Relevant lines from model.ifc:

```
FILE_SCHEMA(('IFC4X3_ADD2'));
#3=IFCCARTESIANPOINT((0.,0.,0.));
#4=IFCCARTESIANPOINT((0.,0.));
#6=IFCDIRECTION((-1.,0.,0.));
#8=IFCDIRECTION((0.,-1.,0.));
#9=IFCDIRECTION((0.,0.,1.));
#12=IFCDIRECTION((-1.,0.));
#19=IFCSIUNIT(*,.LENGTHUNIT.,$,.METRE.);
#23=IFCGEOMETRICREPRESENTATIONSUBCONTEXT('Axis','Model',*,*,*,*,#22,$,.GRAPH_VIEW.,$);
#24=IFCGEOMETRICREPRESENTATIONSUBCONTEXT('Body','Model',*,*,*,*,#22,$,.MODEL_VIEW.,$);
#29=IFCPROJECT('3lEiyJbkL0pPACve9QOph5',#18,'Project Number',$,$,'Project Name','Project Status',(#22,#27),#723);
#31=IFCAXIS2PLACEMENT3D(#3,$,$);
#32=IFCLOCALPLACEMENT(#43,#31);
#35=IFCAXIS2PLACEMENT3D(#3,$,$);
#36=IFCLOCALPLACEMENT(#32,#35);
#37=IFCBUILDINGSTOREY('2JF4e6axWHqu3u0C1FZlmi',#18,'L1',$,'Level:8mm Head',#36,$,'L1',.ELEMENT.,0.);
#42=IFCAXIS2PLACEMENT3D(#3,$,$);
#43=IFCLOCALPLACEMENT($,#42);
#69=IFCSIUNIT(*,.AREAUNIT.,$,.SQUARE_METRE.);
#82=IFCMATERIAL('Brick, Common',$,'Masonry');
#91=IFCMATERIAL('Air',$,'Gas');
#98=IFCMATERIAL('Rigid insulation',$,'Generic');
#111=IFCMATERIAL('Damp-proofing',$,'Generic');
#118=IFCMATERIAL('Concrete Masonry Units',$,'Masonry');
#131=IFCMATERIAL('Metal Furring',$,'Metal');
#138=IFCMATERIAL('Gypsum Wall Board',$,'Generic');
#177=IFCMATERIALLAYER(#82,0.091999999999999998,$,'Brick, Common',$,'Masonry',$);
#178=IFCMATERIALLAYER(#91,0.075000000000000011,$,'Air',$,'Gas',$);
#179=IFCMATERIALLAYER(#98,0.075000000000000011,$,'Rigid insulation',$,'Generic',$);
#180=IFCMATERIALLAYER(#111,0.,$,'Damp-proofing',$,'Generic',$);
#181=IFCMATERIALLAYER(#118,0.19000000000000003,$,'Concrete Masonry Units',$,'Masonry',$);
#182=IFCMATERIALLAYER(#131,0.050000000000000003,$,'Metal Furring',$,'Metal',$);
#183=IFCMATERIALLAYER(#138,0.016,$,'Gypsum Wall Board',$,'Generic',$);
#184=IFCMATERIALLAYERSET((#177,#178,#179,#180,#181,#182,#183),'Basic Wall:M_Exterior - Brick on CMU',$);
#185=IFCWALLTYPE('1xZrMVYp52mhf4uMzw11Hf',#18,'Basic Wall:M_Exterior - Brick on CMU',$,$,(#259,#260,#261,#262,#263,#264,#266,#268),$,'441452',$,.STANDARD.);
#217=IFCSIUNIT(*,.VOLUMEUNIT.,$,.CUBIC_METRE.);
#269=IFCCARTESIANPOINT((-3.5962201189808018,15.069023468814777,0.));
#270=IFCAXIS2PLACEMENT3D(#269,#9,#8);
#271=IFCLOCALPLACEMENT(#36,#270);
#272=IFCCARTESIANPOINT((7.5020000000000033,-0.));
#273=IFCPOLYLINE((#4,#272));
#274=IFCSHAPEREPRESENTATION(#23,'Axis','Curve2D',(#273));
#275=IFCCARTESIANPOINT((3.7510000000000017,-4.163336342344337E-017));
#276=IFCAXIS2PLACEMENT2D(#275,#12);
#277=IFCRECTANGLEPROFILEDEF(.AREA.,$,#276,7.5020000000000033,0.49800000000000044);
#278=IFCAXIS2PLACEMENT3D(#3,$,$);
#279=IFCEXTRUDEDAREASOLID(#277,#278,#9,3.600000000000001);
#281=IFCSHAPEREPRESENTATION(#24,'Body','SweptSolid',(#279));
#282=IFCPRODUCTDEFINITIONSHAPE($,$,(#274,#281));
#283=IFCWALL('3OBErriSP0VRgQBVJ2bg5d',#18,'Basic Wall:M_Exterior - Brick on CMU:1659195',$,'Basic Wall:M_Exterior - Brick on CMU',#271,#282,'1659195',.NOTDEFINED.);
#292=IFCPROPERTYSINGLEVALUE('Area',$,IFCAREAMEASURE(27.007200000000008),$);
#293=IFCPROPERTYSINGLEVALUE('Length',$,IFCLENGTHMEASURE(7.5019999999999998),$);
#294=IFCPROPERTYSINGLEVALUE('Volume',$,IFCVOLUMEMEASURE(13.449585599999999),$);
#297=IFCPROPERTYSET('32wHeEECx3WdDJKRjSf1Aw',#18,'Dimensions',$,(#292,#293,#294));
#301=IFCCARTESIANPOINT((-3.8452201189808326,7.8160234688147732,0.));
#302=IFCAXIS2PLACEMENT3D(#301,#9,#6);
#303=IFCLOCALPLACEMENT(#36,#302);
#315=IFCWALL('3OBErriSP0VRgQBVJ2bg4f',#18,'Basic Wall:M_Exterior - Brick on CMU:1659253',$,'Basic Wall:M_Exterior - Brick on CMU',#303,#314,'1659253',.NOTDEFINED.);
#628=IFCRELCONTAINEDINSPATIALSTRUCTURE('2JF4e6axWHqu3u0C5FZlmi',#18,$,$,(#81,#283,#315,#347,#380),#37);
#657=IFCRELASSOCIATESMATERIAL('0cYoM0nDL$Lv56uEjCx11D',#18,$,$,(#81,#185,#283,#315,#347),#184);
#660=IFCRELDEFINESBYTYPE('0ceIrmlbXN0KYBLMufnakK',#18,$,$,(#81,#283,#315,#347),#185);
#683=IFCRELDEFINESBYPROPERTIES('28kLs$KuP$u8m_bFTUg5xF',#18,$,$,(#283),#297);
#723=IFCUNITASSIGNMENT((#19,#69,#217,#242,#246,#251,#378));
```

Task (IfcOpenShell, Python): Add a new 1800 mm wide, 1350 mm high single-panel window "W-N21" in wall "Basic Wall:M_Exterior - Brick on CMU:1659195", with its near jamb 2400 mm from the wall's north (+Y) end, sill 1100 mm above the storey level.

```python
import numpy as np
import ifcopenshell
import ifcopenshell.api.feature
import ifcopenshell.api.geometry
import ifcopenshell.api.pset
import ifcopenshell.api.root
import ifcopenshell.api.spatial
import ifcopenshell.geom
import ifcopenshell.util.element
import ifcopenshell.util.placement
import ifcopenshell.util.representation
import ifcopenshell.util.shape
import ifcopenshell.util.unit

model = ifcopenshell.open("model.ifc")
unit_scale = ifcopenshell.util.unit.calculate_unit_scale(model)
area_scale = ifcopenshell.util.unit.calculate_unit_scale(model, "AREAUNIT")
volume_scale = ifcopenshell.util.unit.calculate_unit_scale(model, "VOLUMEUNIT")
settings = ifcopenshell.geom.settings()


def volume(element):
    """Net volume in cubic metres, openings subtracted."""
    shape = ifcopenshell.geom.create_shape(settings, element)
    return ifcopenshell.util.shape.get_volume(shape.geometry)


wall = model.by_guid("3OBErriSP0VRgQBVJ2bg5d")
storey = ifcopenshell.util.element.get_container(wall, ifc_class="IfcBuildingStorey")
context = ifcopenshell.util.representation.get_context(model, "Model", "Body", "MODEL_VIEW")
before = volume(wall)

width, height, from_end, sill = 1.8, 1.35, 2.4, 1.1  # metres

# The wall runs along its own X axis, and the end named is its -X end.
wall_shape = ifcopenshell.geom.create_shape(settings, wall)
x, y, z = ifcopenshell.util.shape.get_vertices(wall_shape.geometry).T
start = x.min() + from_end
face, thickness = float(y.min()), float(y.max() - y.min())
wall_matrix = ifcopenshell.util.placement.get_local_placement(wall.ObjectPlacement)
level = ifcopenshell.util.placement.get_local_placement(storey.ObjectPlacement)[2, 3]


def in_wall(x, y):
    """Placement at x, y metres in the wall's axes, at sill height."""
    matrix = wall_matrix.copy()
    matrix[:, 3] = wall_matrix @ np.array([x / unit_scale, y / unit_scale, 0.0, 1.0])
    matrix[2, 3] = level + sill / unit_scale
    return matrix


# Opening: a box that overshoots both wall faces by 50 mm.
opening = ifcopenshell.api.root.create_entity(model, ifc_class="IfcOpeningElement", predefined_type="OPENING")
box = ifcopenshell.api.geometry.add_wall_representation(
    model, context=context, length=width, height=height, thickness=thickness + 0.1
)
ifcopenshell.api.geometry.assign_representation(model, product=opening, representation=box)
ifcopenshell.api.geometry.edit_object_placement(model, product=opening, matrix=in_wall(start, face - 0.05), is_si=False)
ifcopenshell.api.feature.add_feature(model, feature=opening, element=wall)

window = ifcopenshell.api.root.create_entity(model, ifc_class="IfcWindow", name="W-N21", predefined_type="WINDOW")
window.OverallWidth, window.OverallHeight = width / unit_scale, height / unit_scale
window.PartitioningType = "SINGLE_PANEL"
body = ifcopenshell.api.geometry.add_window_representation(
    model,
    context=context,
    overall_width=window.OverallWidth,
    overall_height=window.OverallHeight,
    partition_type="SINGLE_PANEL",
)
ifcopenshell.api.geometry.assign_representation(model, product=window, representation=body)
ifcopenshell.api.spatial.assign_container(model, products=[window], relating_structure=storey)
ifcopenshell.api.feature.add_filling(model, opening=opening, element=window)

# Centre the window in the wall's thickness.
ifcopenshell.api.geometry.edit_object_placement(model, product=window, matrix=in_wall(start, face), is_si=False)
window_shape = ifcopenshell.geom.create_shape(settings, window)
depth = ifcopenshell.util.shape.get_vertices(window_shape.geometry)[:, 1]
offset = face + thickness / 2 - (depth.min() + depth.max()) / 2
ifcopenshell.api.geometry.edit_object_placement(model, product=window, matrix=in_wall(start, offset), is_si=False)

after = volume(wall)

# Update the wall's stored quantities.
pset = model.by_id(ifcopenshell.util.element.get_pset(wall, "Dimensions", should_inherit=False)["id"])
ifcopenshell.api.pset.edit_pset(model, pset=pset, properties={
    "Area": model.create_entity("IfcAreaMeasure", after / thickness / area_scale),
    "Volume": model.create_entity("IfcVolumeMeasure", after / volume_scale),
})

print(f"wall volume {before:.3f} -> {after:.3f} m3")

model.write("model-out.ifc")
```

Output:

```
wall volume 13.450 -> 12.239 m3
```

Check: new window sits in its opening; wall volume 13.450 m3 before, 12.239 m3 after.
